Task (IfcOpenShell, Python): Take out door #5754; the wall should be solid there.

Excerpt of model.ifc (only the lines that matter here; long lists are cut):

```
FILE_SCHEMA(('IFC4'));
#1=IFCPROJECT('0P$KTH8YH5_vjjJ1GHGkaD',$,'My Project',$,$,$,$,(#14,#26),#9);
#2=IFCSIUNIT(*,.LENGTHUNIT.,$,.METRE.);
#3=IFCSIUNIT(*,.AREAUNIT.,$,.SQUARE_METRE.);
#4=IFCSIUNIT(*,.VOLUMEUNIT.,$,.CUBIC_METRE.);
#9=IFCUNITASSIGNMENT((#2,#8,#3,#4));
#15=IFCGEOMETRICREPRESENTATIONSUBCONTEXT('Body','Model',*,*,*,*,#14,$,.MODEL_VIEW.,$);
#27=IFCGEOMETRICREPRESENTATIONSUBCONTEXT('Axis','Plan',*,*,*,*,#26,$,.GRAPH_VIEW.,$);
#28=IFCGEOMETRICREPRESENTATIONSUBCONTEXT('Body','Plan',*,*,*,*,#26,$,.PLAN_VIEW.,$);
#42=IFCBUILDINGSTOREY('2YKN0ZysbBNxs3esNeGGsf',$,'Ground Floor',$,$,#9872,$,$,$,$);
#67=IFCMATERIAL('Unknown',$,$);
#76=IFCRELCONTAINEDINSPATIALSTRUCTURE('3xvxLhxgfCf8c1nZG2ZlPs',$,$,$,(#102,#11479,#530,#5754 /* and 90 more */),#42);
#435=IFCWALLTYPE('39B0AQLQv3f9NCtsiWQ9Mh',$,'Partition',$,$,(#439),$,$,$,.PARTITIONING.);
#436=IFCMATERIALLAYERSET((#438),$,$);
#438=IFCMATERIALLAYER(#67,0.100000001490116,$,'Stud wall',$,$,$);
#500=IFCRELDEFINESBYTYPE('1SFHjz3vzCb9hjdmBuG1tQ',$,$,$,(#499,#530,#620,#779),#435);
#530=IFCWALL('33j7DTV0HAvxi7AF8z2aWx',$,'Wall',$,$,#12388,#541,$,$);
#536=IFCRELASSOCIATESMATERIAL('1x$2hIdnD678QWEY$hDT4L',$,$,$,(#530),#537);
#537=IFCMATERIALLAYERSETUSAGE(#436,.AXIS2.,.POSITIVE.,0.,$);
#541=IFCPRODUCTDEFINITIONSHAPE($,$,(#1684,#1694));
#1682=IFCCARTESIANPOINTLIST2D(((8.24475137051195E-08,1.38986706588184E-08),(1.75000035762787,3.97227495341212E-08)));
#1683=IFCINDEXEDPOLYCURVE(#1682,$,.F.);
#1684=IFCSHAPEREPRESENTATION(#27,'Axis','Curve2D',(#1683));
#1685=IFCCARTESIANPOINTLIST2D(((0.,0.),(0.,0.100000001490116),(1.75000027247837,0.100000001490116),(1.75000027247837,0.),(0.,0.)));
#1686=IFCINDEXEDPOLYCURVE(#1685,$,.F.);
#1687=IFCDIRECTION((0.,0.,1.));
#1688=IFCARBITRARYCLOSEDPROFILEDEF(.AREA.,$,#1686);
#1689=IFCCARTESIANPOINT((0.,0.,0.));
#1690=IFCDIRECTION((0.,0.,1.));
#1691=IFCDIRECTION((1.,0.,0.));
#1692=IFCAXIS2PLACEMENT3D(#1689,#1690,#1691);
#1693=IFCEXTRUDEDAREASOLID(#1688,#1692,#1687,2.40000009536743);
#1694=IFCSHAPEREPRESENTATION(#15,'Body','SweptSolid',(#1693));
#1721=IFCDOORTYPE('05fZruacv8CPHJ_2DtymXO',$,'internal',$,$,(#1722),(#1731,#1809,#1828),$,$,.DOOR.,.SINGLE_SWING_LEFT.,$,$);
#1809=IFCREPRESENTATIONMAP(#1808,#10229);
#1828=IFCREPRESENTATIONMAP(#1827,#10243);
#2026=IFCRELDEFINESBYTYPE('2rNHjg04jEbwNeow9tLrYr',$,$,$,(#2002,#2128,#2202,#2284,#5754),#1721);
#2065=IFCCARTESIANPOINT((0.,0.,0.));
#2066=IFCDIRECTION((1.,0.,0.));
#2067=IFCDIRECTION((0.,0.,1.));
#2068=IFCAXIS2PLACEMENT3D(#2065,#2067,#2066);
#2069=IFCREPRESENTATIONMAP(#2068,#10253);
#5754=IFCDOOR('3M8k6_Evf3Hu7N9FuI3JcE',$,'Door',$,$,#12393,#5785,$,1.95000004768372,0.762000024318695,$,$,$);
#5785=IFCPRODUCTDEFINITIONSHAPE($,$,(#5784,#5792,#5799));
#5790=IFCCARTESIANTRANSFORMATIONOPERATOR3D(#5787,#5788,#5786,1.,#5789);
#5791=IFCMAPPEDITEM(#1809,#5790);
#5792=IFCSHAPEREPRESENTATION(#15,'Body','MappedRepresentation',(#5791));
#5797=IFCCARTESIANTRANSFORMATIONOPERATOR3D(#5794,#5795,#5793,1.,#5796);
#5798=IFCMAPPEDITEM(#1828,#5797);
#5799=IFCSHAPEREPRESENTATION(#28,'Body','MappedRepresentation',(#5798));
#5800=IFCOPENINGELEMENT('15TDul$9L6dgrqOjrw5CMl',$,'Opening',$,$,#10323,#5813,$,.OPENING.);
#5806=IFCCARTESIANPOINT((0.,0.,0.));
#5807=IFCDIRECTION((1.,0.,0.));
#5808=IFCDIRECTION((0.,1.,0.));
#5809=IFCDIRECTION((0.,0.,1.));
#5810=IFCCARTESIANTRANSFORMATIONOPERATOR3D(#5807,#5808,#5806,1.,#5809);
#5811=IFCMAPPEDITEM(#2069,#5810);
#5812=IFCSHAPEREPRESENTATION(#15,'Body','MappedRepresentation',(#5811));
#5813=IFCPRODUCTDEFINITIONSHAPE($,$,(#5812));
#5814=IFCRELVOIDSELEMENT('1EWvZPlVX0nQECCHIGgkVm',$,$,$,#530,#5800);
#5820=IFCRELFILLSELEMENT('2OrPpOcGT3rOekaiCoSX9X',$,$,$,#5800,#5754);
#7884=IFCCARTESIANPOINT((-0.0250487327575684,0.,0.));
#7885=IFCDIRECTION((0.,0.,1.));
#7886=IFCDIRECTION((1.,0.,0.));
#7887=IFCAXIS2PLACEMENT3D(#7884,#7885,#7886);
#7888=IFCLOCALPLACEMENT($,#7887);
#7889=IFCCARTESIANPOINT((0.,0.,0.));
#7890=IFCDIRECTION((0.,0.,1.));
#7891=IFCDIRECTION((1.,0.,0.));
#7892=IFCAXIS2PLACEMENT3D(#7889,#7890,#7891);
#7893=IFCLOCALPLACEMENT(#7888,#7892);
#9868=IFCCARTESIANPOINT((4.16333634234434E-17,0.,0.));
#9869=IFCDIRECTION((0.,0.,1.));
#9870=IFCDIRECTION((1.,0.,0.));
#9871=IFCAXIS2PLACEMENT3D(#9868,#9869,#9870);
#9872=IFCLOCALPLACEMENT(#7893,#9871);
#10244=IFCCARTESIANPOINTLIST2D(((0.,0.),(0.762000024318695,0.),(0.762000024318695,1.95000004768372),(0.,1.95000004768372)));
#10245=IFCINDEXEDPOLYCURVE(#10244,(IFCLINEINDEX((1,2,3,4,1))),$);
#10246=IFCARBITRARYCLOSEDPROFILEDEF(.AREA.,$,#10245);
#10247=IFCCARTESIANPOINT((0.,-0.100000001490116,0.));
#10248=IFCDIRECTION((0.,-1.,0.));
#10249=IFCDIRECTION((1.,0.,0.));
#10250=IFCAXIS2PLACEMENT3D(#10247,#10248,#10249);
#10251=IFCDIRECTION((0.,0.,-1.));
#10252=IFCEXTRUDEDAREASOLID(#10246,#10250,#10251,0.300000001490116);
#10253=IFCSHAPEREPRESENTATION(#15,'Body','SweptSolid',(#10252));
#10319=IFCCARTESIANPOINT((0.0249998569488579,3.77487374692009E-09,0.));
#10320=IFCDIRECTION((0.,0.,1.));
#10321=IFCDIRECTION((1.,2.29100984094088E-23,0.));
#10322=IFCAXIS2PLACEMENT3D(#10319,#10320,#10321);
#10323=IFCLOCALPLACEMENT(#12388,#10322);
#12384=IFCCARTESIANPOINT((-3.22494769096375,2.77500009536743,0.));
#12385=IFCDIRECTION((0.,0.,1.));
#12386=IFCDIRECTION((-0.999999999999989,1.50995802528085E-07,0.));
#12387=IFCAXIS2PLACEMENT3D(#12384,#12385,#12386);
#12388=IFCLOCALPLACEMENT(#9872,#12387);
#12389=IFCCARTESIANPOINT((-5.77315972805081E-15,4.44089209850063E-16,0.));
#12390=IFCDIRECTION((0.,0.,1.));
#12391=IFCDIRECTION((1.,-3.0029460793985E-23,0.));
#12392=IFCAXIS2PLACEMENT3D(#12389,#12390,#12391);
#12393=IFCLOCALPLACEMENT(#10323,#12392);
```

```python
import ifcopenshell
import ifcopenshell.api.feature
import ifcopenshell.api.root
import ifcopenshell.geom
import ifcopenshell.util.shape

model = ifcopenshell.open("model.ifc")
settings = ifcopenshell.geom.settings()


def volume(element):
    """Net volume in cubic metres, openings subtracted."""
    shape = ifcopenshell.geom.create_shape(settings, element)
    return ifcopenshell.util.shape.get_volume(shape.geometry)


door = model.by_guid("3M8k6_Evf3Hu7N9FuI3JcE")
opening = door.FillsVoids[0].RelatingOpeningElement
wall = opening.VoidsElements[0].RelatingBuildingElement
before = volume(wall)

ifcopenshell.api.root.remove_product(model, product=door)
ifcopenshell.api.feature.remove_feature(model, feature=opening)

after = volume(wall)

print(f"wall volume {before:.3f} -> {after:.3f} m3")

model.write("model_updated.ifc")
```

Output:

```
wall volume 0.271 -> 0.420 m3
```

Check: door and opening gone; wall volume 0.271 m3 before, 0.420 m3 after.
